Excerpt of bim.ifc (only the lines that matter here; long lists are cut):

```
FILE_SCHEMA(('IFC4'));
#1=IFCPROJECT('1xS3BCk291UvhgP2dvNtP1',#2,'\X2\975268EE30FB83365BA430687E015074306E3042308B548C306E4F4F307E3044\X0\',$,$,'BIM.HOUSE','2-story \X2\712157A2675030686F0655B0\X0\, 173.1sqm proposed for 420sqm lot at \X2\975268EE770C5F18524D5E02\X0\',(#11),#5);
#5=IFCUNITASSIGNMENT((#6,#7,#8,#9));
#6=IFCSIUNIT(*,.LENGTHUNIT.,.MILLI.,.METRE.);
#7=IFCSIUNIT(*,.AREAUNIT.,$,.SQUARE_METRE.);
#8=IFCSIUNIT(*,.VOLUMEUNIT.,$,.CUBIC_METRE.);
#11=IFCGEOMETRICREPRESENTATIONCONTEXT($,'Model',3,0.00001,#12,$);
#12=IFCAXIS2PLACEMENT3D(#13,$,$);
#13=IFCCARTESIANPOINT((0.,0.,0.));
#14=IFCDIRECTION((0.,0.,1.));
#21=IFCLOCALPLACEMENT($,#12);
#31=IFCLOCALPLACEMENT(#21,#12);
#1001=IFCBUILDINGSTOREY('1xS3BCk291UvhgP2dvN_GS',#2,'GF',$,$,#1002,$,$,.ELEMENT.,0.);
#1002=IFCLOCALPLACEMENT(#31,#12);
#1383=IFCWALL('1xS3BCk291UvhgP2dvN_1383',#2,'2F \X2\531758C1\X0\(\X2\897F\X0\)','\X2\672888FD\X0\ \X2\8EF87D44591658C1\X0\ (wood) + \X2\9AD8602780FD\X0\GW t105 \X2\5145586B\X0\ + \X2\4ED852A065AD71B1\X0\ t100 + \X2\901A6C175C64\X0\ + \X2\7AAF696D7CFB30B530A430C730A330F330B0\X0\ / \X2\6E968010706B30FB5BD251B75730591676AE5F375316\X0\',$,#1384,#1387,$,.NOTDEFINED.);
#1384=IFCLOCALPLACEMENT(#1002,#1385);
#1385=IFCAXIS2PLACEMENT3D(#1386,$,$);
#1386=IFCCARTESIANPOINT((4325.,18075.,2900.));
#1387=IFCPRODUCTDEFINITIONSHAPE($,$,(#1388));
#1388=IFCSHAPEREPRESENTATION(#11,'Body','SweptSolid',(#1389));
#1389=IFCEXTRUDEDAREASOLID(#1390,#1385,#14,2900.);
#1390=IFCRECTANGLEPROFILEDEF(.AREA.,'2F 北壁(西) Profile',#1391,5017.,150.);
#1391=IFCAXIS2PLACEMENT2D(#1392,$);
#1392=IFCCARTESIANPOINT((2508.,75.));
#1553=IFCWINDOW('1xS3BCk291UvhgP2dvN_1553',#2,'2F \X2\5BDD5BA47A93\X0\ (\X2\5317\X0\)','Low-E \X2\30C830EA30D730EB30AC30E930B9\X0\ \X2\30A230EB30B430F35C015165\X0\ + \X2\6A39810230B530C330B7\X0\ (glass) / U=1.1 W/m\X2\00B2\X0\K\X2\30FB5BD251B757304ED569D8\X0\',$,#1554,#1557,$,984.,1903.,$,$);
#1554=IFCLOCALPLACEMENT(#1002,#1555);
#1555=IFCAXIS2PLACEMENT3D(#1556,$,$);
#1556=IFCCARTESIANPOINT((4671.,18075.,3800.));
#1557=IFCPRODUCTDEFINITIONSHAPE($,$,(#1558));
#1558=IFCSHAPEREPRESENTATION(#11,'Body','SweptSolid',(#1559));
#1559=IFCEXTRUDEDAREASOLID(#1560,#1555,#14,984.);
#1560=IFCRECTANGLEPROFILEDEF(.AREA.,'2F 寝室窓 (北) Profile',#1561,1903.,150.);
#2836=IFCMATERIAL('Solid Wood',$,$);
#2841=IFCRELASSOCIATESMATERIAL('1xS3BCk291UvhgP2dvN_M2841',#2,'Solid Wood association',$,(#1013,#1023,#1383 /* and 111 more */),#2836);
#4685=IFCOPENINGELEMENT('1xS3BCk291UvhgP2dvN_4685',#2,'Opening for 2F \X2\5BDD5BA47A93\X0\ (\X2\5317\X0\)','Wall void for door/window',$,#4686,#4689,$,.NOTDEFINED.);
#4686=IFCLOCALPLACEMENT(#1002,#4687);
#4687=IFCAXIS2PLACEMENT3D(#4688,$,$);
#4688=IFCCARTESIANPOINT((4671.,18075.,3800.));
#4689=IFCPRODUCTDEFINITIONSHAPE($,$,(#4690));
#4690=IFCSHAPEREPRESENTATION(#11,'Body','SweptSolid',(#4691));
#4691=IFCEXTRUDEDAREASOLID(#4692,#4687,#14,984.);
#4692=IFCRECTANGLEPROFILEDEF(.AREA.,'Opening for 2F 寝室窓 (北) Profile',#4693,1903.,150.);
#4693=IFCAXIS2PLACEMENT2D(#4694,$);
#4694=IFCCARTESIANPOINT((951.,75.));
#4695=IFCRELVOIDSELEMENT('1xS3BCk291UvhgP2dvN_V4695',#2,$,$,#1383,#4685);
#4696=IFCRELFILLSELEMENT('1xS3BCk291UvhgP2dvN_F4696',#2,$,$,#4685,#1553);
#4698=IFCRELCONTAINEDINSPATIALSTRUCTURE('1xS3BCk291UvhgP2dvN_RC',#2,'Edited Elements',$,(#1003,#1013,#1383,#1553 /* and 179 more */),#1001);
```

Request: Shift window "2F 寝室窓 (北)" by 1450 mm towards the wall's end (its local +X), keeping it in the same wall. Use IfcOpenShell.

```python
import ifcopenshell
import ifcopenshell.api.geometry
import ifcopenshell.util.placement

model = ifcopenshell.open("bim.ifc")

window = model.by_guid("1xS3BCk291UvhgP2dvN_1553")
opening = window.FillsVoids[0].RelatingOpeningElement
wall = opening.VoidsElements[0].RelatingBuildingElement

wall_matrix = ifcopenshell.util.placement.get_local_placement(wall.ObjectPlacement)
shift = wall_matrix[:3, 0] * 1450.0
before = ifcopenshell.util.placement.get_local_placement(window.ObjectPlacement)[:3, 3].copy()

# The window is not placed relative to its opening, so move both.
for product in (opening, window):
    matrix = ifcopenshell.util.placement.get_local_placement(product.ObjectPlacement)
    matrix[:3, 3] += shift
    ifcopenshell.api.geometry.edit_object_placement(model, product=product, matrix=matrix, is_si=False)

after = ifcopenshell.util.placement.get_local_placement(window.ObjectPlacement)[:3, 3]
print("window moved by", (after - before).round(3) + 0.0)

model.write("bim_v2.ifc")
```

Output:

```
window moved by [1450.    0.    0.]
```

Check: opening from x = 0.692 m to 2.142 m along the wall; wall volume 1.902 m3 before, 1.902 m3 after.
